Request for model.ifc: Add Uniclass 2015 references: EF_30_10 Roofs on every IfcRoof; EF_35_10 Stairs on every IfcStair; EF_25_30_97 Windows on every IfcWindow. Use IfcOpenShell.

First a look at what the model holds.

```python
import ifcopenshell

model = ifcopenshell.open("model.ifc")
print(model.schema)
print("classifications:", [c.Name for c in model.by_type("IfcClassification")])
for ifc_class in ("IfcDoor", "IfcRoof", "IfcStair", "IfcWall", "IfcWindow"):
    print(ifc_class, len(model.by_type(ifc_class)))
```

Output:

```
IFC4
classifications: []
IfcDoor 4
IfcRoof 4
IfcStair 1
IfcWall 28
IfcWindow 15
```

```python
import ifcopenshell
import ifcopenshell.api.classification

model = ifcopenshell.open("model.ifc")

system = ifcopenshell.api.classification.add_classification(model, classification="Uniclass 2015")

codes = {
    "IfcRoof": ("EF_30_10", "Roofs"),
    "IfcStair": ("EF_35_10", "Stairs"),
    "IfcWindow": ("EF_25_30_97", "Windows"),
}
for ifc_class, (code, name) in codes.items():
    products = model.by_type(ifc_class)
    ifcopenshell.api.classification.add_reference(
        model, products=products, classification=system, identification=code, name=name
    )
    print(code, len(products))

model.write("model-out.ifc")
```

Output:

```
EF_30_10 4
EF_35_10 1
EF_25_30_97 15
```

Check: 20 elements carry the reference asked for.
